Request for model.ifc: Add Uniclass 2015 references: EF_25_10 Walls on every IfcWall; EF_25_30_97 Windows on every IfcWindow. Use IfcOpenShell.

First a look at what the model holds.

```python
import ifcopenshell

model = ifcopenshell.open("model.ifc")
print(model.schema)
print("classifications:", [c.Name for c in model.by_type("IfcClassification")])
for ifc_class in ("IfcDoor", "IfcRoof", "IfcStair", "IfcWall", "IfcWindow"):
    print(ifc_class, len(model.by_type(ifc_class)))
```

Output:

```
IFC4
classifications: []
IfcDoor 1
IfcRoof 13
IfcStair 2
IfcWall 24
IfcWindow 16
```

```python
import ifcopenshell
import ifcopenshell.api.classification

model = ifcopenshell.open("model.ifc")

system = ifcopenshell.api.classification.add_classification(model, classification="Uniclass 2015")

codes = {
    "IfcWall": ("EF_25_10", "Walls"),
    "IfcWindow": ("EF_25_30_97", "Windows"),
}
for ifc_class, (code, name) in codes.items():
    products = model.by_type(ifc_class)
    ifcopenshell.api.classification.add_reference(
        model, products=products, classification=system, identification=code, name=name
    )
    print(code, len(products))

model.write("model_updated.ifc")
```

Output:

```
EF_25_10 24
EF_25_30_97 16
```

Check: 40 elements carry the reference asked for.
